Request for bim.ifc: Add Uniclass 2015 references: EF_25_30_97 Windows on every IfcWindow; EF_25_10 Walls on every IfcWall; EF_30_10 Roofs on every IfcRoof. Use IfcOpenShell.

First a look at what the model holds.

```python
import ifcopenshell

model = ifcopenshell.open("bim.ifc")
print(model.schema)
print("classifications:", [c.Name for c in model.by_type("IfcClassification")])
for ifc_class in ("IfcDoor", "IfcRoof", "IfcStair", "IfcWall", "IfcWindow"):
    print(ifc_class, len(model.by_type(ifc_class)))
```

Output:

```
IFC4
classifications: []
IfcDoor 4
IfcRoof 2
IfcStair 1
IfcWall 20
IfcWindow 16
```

```python
import ifcopenshell
import ifcopenshell.api.classification

model = ifcopenshell.open("bim.ifc")

system = ifcopenshell.api.classification.add_classification(model, classification="Uniclass 2015")

codes = {
    "IfcWindow": ("EF_25_30_97", "Windows"),
    "IfcWall": ("EF_25_10", "Walls"),
    "IfcRoof": ("EF_30_10", "Roofs"),
}
for ifc_class, (code, name) in codes.items():
    products = model.by_type(ifc_class)
    ifcopenshell.api.classification.add_reference(
        model, products=products, classification=system, identification=code, name=name
    )
    print(code, len(products))

model.write("bim_edited.ifc")
```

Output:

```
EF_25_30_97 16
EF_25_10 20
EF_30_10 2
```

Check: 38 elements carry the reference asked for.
